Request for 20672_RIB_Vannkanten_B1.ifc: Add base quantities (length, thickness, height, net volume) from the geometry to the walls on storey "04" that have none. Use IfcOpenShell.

First a look at what the model holds.

```python
import ifcopenshell
import ifcopenshell.util.element
import ifcopenshell.util.unit

model = ifcopenshell.open("20672_RIB_Vannkanten_B1.ifc")
print(model.schema)
for unit_type in ("LENGTHUNIT", "AREAUNIT", "VOLUMEUNIT"):
    print(unit_type, ifcopenshell.util.unit.calculate_unit_scale(model, unit_type))
storey = next(s for s in model.by_type("IfcBuildingStorey") if s.Name == "04")
walls = [e for e in ifcopenshell.util.element.get_decomposition(storey) if e.is_a("IfcWall")]
for e in sorted(walls, key=lambda e: e.id()):
    print(e.id(), e.is_a(), e.Name, list(ifcopenshell.util.element.get_psets(e, qtos_only=True)), sep=" | ")
```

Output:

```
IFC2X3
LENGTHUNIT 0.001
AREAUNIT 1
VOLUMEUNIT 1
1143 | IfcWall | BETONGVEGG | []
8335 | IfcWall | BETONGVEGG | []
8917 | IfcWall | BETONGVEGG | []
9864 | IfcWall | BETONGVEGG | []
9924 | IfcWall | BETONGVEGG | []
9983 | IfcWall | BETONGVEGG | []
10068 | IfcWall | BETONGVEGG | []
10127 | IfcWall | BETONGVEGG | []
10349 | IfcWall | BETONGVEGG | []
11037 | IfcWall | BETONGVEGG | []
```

```python
import ifcopenshell
import ifcopenshell.api.pset
import ifcopenshell.geom
import ifcopenshell.util.element
import ifcopenshell.util.shape
import ifcopenshell.util.unit

model = ifcopenshell.open("20672_RIB_Vannkanten_B1.ifc")
unit_scale = ifcopenshell.util.unit.calculate_unit_scale(model)
volume_scale = ifcopenshell.util.unit.calculate_unit_scale(model, "VOLUMEUNIT")
settings = ifcopenshell.geom.settings()

storey = next(s for s in model.by_type("IfcBuildingStorey") if s.Name == "04")
walls = [e for e in ifcopenshell.util.element.get_decomposition(storey) if e.is_a("IfcWall")]

for e in sorted(walls, key=lambda e: e.id()):
    if ifcopenshell.util.element.get_psets(e, qtos_only=True, should_inherit=False):
        continue
    # Geometry comes back in metres, in the element's own axes.
    shape = ifcopenshell.geom.create_shape(settings, e)
    values = {
        "Length": ifcopenshell.util.shape.get_x(shape.geometry) / unit_scale,
        "Width": ifcopenshell.util.shape.get_y(shape.geometry) / unit_scale,
        "Height": ifcopenshell.util.shape.get_z(shape.geometry) / unit_scale,
        "NetVolume": ifcopenshell.util.shape.get_volume(shape.geometry) / volume_scale,
    }
    qto = ifcopenshell.api.pset.add_qto(model, product=e, name="BaseQuantities")
    ifcopenshell.api.pset.edit_qto(model, qto=qto, properties=values)
    print(e.id(), {k: round(v, 3) for k, v in values.items()})

model.write("20672_RIB_Vannkanten_B1_updated.ifc")
```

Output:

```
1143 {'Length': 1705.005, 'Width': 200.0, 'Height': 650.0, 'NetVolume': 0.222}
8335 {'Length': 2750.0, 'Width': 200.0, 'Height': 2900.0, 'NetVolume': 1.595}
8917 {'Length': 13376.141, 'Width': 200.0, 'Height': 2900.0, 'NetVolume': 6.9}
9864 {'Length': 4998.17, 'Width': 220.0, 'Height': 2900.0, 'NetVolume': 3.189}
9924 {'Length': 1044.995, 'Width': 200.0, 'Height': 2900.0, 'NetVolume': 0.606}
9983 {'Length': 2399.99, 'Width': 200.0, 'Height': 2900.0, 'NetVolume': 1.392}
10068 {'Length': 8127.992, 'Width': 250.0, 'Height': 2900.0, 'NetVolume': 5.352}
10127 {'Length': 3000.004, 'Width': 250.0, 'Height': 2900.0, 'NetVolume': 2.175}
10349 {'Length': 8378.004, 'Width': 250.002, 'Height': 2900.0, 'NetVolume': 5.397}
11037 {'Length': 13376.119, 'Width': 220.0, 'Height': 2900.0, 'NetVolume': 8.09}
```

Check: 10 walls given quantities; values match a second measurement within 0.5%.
